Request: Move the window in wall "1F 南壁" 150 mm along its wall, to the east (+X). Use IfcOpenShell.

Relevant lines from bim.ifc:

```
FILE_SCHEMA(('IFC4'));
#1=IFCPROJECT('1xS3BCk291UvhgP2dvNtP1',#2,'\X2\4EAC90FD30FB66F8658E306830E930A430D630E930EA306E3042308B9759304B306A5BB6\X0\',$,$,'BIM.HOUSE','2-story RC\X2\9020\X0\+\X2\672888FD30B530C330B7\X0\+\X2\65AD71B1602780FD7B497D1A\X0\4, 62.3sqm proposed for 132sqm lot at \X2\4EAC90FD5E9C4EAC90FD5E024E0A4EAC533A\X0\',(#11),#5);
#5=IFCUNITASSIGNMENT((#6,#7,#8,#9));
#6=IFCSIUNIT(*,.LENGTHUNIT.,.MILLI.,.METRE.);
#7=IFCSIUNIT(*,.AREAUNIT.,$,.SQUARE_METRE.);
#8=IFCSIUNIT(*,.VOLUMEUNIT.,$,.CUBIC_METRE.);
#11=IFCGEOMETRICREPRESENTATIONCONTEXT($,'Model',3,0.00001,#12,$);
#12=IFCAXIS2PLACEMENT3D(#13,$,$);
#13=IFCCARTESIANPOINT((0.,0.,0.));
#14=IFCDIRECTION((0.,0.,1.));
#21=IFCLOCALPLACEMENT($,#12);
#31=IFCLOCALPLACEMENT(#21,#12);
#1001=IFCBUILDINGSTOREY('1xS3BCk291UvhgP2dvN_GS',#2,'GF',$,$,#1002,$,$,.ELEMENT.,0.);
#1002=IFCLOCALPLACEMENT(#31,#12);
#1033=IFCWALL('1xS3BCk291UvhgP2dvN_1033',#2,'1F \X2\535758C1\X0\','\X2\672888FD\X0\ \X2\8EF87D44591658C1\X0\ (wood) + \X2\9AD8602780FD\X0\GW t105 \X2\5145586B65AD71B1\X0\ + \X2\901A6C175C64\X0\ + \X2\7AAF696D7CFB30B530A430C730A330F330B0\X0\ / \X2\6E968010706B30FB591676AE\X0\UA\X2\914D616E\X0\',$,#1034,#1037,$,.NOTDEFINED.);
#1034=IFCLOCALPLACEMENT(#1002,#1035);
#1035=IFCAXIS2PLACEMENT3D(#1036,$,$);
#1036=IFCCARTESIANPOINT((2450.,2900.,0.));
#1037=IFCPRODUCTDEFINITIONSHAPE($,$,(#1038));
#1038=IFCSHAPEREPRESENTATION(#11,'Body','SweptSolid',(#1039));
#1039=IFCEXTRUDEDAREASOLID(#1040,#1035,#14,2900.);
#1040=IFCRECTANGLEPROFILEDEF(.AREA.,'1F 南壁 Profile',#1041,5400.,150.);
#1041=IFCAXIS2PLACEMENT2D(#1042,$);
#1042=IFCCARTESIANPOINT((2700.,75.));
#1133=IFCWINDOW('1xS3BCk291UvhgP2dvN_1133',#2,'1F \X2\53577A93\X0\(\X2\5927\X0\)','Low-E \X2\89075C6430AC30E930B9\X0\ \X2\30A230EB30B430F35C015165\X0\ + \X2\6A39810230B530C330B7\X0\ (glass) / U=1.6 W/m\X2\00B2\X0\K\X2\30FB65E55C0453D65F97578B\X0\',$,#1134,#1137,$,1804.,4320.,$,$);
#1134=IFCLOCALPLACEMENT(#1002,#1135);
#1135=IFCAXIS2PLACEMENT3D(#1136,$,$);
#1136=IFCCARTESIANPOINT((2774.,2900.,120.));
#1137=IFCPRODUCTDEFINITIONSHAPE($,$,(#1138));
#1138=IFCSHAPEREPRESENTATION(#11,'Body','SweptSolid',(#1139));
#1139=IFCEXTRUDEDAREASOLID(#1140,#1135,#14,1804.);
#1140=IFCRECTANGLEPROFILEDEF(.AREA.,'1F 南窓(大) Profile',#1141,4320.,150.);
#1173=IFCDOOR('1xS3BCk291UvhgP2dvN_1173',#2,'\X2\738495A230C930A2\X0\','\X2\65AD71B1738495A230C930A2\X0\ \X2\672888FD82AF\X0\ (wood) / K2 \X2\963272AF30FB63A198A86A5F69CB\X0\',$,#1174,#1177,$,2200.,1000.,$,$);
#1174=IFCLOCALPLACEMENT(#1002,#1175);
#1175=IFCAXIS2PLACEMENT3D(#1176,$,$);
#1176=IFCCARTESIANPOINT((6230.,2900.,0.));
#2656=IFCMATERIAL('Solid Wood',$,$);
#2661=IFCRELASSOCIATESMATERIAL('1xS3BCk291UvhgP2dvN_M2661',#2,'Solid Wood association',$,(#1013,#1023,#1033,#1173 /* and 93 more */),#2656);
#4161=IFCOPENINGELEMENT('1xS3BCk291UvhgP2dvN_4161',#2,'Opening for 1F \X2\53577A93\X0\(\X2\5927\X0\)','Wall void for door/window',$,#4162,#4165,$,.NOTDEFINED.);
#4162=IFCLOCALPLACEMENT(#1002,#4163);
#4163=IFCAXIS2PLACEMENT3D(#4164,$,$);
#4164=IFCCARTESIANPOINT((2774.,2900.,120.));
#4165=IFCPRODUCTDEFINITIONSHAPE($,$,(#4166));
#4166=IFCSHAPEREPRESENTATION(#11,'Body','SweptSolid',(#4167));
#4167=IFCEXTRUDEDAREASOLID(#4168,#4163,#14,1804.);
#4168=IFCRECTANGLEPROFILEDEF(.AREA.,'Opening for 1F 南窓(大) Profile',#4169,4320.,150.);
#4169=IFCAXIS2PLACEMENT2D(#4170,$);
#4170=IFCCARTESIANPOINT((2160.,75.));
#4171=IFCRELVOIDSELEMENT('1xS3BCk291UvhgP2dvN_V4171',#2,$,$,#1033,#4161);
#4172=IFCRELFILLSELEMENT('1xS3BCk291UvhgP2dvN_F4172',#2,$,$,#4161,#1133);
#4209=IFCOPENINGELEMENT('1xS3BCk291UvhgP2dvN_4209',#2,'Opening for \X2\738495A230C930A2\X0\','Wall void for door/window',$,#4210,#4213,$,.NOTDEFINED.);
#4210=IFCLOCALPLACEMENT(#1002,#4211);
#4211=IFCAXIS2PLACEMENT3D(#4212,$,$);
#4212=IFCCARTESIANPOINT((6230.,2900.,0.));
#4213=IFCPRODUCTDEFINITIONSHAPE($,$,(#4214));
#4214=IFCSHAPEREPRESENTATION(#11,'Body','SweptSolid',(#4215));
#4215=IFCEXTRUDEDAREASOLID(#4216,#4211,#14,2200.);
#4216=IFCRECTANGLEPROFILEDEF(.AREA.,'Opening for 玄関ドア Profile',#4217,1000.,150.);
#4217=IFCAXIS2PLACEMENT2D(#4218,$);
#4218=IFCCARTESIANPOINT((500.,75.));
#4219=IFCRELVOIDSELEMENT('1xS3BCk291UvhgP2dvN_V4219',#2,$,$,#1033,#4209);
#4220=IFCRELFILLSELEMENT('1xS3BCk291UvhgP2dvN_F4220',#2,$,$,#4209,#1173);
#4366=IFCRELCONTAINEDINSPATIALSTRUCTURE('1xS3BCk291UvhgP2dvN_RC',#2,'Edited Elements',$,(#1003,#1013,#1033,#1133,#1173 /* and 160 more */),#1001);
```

```python
import ifcopenshell
import ifcopenshell.api.geometry
import ifcopenshell.util.placement
import ifcopenshell.util.unit

model = ifcopenshell.open("bim.ifc")
unit_scale = ifcopenshell.util.unit.calculate_unit_scale(model)

window = model.by_guid("1xS3BCk291UvhgP2dvN_1133")
opening = window.FillsVoids[0].RelatingOpeningElement
wall = opening.VoidsElements[0].RelatingBuildingElement

wall_matrix = ifcopenshell.util.placement.get_local_placement(wall.ObjectPlacement)
shift = wall_matrix[:3, 0] * 0.15 / unit_scale
before = ifcopenshell.util.placement.get_local_placement(window.ObjectPlacement)[:3, 3].copy()

# The window is not placed relative to its opening, so move both.
for product in (opening, window):
    matrix = ifcopenshell.util.placement.get_local_placement(product.ObjectPlacement)
    matrix[:3, 3] += shift
    ifcopenshell.api.geometry.edit_object_placement(model, product=product, matrix=matrix, is_si=False)

after = ifcopenshell.util.placement.get_local_placement(window.ObjectPlacement)[:3, 3]
print("window moved by", (after - before).round(3) + 0.0)

model.write("bim_edited.ifc")
```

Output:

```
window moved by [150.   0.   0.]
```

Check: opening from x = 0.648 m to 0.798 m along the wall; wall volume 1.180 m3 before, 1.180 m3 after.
